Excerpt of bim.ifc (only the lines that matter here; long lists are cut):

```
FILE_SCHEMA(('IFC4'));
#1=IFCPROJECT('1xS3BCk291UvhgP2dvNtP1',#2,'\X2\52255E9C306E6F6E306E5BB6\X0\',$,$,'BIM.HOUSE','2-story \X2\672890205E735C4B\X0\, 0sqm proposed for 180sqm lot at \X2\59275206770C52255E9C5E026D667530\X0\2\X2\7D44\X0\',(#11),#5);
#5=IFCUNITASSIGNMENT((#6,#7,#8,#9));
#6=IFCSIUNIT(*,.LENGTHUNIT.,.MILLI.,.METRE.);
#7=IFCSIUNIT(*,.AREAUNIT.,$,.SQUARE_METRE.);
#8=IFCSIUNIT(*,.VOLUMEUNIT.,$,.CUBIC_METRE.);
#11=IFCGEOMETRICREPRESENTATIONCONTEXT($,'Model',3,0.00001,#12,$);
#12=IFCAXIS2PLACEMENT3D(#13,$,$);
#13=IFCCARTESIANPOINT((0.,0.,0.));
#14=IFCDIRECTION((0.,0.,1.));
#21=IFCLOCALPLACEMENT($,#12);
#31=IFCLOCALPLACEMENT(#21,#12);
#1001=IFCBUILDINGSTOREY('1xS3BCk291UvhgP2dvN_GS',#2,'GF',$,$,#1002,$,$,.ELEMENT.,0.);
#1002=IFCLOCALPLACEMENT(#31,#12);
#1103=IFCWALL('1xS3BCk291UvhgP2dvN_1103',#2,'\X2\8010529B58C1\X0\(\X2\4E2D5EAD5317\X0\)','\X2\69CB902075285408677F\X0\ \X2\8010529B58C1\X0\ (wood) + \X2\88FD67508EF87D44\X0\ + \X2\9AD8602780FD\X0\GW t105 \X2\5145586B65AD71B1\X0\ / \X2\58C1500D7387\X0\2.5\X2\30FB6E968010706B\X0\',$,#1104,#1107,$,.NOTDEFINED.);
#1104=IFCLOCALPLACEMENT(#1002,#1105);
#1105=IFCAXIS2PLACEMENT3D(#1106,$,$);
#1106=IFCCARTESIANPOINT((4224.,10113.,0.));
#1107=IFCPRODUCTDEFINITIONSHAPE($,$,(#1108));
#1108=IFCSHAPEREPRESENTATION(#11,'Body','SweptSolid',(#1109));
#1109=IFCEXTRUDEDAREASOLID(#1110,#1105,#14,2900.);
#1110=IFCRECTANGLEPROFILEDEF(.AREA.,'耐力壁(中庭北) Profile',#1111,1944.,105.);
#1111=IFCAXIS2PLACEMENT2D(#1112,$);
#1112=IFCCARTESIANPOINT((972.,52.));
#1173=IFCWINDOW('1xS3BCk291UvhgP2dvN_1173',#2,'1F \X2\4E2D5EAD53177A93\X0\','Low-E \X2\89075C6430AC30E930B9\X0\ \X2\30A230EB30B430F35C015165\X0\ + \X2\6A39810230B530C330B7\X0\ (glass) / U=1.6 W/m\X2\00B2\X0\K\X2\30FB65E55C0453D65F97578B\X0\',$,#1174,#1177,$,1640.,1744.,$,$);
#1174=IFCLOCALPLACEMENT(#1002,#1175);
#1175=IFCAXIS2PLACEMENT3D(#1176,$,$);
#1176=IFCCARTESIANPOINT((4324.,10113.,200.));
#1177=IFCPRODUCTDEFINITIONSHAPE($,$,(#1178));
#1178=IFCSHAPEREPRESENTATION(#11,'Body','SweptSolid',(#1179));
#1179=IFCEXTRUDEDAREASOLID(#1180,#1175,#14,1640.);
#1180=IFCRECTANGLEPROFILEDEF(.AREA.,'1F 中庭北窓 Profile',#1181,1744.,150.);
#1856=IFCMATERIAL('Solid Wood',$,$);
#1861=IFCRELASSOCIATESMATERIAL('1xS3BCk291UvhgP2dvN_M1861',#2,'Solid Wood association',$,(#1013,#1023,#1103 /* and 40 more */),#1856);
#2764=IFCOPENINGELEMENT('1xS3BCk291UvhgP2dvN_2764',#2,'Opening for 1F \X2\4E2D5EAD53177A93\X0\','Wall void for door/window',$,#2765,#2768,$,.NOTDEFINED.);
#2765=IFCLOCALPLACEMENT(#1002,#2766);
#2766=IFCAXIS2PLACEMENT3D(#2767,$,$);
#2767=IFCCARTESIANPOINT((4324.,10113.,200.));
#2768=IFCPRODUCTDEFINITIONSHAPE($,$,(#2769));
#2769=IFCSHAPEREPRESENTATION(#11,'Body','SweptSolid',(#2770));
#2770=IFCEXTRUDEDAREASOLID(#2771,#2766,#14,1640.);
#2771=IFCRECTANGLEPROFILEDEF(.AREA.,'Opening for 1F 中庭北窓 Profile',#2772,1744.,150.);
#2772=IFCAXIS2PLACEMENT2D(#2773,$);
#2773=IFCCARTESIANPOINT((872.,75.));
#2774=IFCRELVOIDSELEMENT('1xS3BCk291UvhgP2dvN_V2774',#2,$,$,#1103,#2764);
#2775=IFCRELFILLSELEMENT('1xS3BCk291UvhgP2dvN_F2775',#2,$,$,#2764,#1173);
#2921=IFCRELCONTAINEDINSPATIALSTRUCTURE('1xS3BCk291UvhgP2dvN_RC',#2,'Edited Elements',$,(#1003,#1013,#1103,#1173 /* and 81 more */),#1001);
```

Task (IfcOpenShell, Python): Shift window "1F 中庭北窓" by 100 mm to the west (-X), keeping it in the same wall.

```python
import ifcopenshell
import ifcopenshell.api.geometry
import ifcopenshell.util.placement

model = ifcopenshell.open("bim.ifc")

window = model.by_guid("1xS3BCk291UvhgP2dvN_1173")
opening = window.FillsVoids[0].RelatingOpeningElement
wall = opening.VoidsElements[0].RelatingBuildingElement

wall_matrix = ifcopenshell.util.placement.get_local_placement(wall.ObjectPlacement)
shift = wall_matrix[:3, 0] * -100.0
before = ifcopenshell.util.placement.get_local_placement(window.ObjectPlacement)[:3, 3].copy()

# The window is not placed relative to its opening, so move both.
for product in (opening, window):
    matrix = ifcopenshell.util.placement.get_local_placement(product.ObjectPlacement)
    matrix[:3, 3] += shift
    ifcopenshell.api.geometry.edit_object_placement(model, product=product, matrix=matrix, is_si=False)

after = ifcopenshell.util.placement.get_local_placement(window.ObjectPlacement)[:3, 3]
print("window moved by", (after - before).round(3) + 0.0)

model.write("bim_v2.ifc")
```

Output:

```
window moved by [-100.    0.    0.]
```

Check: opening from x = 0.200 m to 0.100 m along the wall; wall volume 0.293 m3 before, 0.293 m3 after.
